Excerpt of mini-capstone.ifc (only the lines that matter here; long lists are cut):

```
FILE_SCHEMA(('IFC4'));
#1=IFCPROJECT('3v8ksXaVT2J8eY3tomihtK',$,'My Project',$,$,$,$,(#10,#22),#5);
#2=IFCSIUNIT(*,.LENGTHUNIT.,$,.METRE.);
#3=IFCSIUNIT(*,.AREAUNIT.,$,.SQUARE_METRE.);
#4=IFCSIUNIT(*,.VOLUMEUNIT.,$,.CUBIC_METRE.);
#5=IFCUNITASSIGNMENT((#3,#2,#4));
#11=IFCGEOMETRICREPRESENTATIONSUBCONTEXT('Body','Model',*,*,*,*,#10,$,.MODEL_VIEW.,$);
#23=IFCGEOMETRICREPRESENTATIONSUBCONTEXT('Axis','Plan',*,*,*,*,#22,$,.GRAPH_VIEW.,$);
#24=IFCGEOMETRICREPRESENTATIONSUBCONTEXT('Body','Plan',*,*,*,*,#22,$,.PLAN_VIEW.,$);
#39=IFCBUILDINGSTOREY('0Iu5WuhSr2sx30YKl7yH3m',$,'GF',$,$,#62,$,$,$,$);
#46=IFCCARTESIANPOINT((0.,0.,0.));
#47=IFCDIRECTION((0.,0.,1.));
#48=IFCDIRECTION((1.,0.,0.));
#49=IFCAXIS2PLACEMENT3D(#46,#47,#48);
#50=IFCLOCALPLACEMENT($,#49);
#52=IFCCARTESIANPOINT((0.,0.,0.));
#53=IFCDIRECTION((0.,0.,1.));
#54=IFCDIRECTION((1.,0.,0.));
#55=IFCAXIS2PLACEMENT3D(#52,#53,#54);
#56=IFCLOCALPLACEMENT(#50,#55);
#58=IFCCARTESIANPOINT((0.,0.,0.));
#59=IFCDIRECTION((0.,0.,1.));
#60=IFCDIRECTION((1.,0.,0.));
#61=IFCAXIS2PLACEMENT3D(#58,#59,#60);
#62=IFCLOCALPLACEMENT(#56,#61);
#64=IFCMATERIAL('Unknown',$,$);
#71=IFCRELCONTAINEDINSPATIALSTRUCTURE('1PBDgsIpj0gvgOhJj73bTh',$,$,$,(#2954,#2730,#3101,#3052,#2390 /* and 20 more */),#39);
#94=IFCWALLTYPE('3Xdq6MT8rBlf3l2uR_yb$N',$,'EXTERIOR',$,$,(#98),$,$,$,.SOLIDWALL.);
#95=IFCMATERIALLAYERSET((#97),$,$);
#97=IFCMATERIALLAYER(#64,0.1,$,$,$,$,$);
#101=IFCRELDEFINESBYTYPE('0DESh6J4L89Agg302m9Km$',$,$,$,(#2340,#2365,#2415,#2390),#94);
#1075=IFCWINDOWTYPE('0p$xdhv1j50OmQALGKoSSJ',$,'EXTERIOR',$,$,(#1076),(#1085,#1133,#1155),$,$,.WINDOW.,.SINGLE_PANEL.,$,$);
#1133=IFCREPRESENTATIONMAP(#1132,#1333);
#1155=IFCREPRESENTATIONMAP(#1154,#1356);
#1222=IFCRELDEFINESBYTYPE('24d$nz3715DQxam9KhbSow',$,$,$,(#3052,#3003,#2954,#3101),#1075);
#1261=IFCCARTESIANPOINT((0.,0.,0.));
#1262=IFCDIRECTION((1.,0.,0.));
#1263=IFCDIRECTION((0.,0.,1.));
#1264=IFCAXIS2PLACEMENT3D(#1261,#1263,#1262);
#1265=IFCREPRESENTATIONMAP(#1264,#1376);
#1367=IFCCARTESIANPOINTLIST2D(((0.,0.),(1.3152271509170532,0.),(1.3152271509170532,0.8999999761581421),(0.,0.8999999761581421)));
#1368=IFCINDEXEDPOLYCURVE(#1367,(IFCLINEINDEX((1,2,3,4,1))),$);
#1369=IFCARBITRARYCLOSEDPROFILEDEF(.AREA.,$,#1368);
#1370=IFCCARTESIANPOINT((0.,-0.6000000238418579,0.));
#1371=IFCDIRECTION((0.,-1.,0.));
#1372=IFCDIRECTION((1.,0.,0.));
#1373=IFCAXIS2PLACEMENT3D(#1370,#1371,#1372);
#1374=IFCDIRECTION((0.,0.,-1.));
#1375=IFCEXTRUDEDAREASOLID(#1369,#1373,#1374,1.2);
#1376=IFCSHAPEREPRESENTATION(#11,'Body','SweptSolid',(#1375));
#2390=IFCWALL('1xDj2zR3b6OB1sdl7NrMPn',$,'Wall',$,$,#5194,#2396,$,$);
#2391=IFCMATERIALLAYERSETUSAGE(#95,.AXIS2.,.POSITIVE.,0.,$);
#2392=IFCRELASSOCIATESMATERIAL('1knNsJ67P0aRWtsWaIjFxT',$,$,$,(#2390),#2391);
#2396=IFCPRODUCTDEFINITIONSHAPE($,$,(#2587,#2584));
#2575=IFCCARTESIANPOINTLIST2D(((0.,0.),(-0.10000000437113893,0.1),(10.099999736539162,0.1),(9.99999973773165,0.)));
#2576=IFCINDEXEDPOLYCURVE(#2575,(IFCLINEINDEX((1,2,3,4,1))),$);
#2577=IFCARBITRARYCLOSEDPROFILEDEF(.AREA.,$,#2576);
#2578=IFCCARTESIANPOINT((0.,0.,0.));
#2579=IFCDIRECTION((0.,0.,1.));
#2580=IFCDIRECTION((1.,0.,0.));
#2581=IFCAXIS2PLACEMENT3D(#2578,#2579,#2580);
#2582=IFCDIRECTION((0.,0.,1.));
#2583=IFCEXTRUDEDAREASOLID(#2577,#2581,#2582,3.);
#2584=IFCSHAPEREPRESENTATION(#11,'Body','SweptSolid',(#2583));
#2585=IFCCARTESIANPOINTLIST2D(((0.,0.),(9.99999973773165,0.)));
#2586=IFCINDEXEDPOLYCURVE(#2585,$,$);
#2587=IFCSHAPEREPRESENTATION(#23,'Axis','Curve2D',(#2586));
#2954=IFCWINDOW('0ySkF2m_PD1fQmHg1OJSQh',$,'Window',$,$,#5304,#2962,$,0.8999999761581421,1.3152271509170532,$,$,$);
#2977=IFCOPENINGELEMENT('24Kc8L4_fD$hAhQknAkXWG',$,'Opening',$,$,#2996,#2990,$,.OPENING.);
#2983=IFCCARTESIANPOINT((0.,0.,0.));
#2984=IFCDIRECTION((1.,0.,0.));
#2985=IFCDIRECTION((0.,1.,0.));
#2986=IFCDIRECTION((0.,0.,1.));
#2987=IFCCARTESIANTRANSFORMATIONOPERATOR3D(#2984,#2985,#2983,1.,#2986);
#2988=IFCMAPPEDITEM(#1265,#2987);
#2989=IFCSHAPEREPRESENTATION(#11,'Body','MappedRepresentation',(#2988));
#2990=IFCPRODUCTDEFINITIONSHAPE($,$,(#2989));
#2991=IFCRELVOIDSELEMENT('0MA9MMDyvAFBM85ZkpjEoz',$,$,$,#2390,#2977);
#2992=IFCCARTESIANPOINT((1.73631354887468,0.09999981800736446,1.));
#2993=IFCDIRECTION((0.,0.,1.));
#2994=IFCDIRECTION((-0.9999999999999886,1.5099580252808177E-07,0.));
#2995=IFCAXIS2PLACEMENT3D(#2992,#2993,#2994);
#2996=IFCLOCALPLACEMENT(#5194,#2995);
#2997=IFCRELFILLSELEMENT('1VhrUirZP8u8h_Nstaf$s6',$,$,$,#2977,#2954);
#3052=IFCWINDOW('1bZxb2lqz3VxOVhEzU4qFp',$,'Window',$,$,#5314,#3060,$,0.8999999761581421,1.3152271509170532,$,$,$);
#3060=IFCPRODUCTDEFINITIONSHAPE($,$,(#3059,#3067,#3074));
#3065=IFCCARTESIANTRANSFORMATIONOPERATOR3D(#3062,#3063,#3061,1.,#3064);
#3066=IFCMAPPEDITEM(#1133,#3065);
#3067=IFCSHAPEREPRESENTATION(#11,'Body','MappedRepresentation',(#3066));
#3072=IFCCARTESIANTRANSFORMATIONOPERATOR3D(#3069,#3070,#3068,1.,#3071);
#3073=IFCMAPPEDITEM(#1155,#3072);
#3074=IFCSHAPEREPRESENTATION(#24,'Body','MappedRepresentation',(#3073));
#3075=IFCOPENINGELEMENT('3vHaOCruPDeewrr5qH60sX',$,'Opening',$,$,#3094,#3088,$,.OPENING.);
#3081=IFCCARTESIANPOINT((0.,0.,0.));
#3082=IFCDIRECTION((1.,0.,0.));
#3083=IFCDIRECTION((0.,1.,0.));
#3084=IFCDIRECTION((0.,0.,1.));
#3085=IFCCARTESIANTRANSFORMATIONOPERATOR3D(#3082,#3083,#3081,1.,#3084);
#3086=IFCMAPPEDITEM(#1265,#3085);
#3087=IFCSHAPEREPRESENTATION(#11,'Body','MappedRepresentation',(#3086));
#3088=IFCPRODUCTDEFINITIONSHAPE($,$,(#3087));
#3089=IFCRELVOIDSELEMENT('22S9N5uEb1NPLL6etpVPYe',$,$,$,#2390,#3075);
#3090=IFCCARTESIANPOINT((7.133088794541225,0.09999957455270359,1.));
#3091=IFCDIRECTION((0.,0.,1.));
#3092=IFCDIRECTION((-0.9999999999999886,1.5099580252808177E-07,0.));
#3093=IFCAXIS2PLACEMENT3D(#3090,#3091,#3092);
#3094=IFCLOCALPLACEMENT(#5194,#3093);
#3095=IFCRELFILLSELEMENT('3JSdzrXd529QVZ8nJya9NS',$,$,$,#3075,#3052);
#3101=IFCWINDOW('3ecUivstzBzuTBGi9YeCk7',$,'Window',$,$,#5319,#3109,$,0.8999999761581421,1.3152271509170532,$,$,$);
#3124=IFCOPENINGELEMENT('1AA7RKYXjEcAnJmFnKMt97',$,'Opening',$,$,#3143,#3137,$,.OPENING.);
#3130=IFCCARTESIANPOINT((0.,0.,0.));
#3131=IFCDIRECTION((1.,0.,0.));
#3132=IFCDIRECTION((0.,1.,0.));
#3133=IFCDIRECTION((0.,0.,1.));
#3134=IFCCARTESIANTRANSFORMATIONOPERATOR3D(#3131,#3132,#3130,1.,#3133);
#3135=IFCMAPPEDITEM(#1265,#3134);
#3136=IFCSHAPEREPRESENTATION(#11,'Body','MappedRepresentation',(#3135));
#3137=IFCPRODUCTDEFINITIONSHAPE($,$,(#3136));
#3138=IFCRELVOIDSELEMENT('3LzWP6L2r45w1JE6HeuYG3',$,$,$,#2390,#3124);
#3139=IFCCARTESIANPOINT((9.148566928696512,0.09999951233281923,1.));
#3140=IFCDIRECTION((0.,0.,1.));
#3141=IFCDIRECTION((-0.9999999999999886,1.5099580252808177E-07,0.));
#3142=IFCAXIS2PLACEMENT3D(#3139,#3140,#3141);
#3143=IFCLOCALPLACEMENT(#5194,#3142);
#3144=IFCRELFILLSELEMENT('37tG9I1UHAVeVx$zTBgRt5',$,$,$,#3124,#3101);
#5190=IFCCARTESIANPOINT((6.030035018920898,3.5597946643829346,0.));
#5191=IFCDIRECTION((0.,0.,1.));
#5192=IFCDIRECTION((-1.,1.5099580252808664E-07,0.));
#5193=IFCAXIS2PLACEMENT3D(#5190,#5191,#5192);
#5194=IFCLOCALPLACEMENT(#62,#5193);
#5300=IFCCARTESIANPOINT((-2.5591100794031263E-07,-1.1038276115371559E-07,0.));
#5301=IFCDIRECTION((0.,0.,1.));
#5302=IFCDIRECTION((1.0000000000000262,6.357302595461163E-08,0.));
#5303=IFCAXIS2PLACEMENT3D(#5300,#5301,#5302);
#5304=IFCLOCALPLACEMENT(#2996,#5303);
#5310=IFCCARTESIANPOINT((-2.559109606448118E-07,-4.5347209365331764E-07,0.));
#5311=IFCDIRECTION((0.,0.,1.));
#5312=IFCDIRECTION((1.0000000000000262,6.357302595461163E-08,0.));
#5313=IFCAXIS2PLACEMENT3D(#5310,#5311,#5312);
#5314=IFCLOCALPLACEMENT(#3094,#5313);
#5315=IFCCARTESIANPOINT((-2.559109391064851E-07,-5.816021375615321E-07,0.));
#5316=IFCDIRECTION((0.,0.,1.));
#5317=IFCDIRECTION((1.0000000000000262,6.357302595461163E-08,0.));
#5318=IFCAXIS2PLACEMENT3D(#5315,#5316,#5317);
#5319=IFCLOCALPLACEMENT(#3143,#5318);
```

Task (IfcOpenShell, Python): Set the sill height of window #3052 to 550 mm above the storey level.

```python
import numpy as np
import ifcopenshell
import ifcopenshell.api.geometry
import ifcopenshell.geom
import ifcopenshell.util.element
import ifcopenshell.util.placement
import ifcopenshell.util.shape
import ifcopenshell.util.unit

model = ifcopenshell.open("mini-capstone.ifc")
unit_scale = ifcopenshell.util.unit.calculate_unit_scale(model)

window = model.by_guid("1bZxb2lqz3VxOVhEzU4qFp")
opening = window.FillsVoids[0].RelatingOpeningElement
storey = ifcopenshell.util.element.get_container(window, ifc_class="IfcBuildingStorey")
level = ifcopenshell.util.placement.get_local_placement(storey.ObjectPlacement)[2, 3]

# The opening's origin need not be at the sill, so measure its lowest point.
shape = ifcopenshell.geom.create_shape(ifcopenshell.geom.settings(), opening)
bottom = ifcopenshell.util.shape.get_shape_bottom_elevation(shape, shape.geometry) / unit_scale
dz = level + 0.55 / unit_scale - bottom

shift = np.array([0.0, 0.0, dz])
# The window is placed relative to its opening, so it follows when the opening moves.
matrix = ifcopenshell.util.placement.get_local_placement(opening.ObjectPlacement)
matrix[:3, 3] += shift
ifcopenshell.api.geometry.edit_object_placement(
    model, product=opening, matrix=matrix, is_si=False, should_transform_children=True
)

print(f"moved by {dz * unit_scale:+.3f} m")

model.write("mini-capstone-out.ifc")
```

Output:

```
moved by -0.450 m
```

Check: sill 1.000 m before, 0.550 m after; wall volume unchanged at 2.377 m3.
